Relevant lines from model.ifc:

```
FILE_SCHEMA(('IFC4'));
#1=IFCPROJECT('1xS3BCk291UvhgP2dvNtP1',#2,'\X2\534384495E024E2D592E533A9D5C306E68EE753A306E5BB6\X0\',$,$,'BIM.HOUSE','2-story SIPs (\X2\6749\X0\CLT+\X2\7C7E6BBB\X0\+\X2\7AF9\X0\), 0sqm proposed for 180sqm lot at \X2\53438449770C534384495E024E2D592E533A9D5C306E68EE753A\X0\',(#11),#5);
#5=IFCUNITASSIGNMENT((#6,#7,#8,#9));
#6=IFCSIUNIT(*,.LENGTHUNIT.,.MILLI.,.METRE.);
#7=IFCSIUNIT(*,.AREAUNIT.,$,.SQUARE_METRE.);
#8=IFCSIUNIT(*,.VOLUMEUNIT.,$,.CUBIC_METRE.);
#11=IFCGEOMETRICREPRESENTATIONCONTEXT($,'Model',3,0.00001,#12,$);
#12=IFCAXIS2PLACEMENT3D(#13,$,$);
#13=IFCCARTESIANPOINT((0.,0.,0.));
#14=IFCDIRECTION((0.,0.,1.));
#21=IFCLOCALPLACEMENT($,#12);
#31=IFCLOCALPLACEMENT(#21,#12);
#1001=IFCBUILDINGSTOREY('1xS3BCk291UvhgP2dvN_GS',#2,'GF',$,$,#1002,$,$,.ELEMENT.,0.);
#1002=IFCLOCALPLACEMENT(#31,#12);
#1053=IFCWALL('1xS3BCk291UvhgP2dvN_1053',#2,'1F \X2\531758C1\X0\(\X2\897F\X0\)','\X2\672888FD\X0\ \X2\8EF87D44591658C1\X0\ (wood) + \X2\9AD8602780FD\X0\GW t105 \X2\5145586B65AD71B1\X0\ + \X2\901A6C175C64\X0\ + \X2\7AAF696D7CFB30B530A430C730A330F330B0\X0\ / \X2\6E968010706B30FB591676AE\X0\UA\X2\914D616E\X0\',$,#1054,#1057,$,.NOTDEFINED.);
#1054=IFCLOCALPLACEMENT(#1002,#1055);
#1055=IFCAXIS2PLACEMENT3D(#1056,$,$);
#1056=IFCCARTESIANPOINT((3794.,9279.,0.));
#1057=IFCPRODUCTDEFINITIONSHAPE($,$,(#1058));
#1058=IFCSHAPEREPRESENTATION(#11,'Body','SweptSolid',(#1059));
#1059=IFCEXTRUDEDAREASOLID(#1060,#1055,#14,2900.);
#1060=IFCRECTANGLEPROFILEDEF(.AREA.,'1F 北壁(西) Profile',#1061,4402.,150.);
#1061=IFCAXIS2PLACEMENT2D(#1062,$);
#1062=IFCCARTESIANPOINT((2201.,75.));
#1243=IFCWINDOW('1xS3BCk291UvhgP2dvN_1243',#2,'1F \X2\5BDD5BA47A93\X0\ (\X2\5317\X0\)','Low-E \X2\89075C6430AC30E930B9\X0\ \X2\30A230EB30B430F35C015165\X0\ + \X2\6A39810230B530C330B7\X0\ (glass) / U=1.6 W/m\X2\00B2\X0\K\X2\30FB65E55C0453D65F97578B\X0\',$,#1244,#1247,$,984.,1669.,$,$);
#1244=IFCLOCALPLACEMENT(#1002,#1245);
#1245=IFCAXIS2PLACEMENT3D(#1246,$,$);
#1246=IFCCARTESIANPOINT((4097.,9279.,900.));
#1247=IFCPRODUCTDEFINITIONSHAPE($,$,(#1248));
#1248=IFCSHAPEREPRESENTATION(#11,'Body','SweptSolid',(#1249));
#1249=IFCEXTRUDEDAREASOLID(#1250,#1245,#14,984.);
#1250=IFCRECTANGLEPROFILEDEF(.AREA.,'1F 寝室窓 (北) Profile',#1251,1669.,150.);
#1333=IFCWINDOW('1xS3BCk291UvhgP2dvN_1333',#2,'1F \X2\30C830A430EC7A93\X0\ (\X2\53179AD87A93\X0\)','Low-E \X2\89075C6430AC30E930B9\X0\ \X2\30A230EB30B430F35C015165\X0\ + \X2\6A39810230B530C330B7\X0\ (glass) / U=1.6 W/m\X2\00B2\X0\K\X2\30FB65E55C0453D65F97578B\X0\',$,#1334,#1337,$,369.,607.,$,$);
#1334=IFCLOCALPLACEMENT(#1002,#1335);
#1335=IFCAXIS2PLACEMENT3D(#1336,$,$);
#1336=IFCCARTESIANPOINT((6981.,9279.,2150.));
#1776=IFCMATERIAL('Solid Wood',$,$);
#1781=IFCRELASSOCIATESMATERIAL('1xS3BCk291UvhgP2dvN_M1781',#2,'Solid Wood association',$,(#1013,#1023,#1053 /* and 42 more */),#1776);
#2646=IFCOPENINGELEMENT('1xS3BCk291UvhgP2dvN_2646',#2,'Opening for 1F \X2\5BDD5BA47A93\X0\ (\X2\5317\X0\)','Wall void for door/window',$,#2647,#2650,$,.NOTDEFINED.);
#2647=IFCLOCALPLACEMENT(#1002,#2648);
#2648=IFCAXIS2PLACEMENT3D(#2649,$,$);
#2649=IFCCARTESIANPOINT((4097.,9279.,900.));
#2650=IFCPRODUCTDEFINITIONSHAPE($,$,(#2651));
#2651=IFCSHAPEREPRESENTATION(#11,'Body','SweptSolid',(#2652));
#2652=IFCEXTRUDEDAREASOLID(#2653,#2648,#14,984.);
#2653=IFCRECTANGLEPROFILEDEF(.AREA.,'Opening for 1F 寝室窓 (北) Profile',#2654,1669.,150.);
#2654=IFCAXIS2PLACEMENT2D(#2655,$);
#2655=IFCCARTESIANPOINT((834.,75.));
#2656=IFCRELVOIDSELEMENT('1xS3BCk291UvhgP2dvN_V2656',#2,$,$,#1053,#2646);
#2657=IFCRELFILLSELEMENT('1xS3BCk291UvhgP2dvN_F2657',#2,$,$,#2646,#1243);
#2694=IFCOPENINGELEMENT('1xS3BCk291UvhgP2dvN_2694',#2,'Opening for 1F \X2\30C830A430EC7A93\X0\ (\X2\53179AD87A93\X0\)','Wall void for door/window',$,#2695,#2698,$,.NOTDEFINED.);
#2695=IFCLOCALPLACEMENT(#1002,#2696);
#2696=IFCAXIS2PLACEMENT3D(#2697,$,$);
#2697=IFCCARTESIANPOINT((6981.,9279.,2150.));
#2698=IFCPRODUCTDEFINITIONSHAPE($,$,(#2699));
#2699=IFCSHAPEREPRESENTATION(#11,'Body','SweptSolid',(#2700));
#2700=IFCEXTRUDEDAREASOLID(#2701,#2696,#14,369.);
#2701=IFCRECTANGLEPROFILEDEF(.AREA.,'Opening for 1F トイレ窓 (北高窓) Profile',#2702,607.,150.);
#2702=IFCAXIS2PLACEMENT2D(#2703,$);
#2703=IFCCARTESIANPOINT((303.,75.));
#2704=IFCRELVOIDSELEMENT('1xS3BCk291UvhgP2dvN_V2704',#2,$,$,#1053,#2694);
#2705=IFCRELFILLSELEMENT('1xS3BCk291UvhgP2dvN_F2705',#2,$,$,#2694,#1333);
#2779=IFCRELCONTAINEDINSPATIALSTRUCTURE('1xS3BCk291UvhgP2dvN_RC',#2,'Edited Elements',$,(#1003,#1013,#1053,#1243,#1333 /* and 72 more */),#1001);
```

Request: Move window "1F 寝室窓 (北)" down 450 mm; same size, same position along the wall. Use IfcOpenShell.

```python
import numpy as np
import ifcopenshell
import ifcopenshell.api.geometry
import ifcopenshell.util.placement
import ifcopenshell.util.unit

model = ifcopenshell.open("model.ifc")
unit_scale = ifcopenshell.util.unit.calculate_unit_scale(model)

window = model.by_id(1243)
opening = window.FillsVoids[0].RelatingOpeningElement
dz = -0.45 / unit_scale

shift = np.array([0.0, 0.0, dz])
# The window is not placed relative to its opening, so move both.
for product in (opening, window):
    matrix = ifcopenshell.util.placement.get_local_placement(product.ObjectPlacement)
    matrix[:3, 3] += shift
    ifcopenshell.api.geometry.edit_object_placement(model, product=product, matrix=matrix, is_si=False)

print(f"moved by {dz * unit_scale:+.3f} m")

model.write("model_rev.ifc")
```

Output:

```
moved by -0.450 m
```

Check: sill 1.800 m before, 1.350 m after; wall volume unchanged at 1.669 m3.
